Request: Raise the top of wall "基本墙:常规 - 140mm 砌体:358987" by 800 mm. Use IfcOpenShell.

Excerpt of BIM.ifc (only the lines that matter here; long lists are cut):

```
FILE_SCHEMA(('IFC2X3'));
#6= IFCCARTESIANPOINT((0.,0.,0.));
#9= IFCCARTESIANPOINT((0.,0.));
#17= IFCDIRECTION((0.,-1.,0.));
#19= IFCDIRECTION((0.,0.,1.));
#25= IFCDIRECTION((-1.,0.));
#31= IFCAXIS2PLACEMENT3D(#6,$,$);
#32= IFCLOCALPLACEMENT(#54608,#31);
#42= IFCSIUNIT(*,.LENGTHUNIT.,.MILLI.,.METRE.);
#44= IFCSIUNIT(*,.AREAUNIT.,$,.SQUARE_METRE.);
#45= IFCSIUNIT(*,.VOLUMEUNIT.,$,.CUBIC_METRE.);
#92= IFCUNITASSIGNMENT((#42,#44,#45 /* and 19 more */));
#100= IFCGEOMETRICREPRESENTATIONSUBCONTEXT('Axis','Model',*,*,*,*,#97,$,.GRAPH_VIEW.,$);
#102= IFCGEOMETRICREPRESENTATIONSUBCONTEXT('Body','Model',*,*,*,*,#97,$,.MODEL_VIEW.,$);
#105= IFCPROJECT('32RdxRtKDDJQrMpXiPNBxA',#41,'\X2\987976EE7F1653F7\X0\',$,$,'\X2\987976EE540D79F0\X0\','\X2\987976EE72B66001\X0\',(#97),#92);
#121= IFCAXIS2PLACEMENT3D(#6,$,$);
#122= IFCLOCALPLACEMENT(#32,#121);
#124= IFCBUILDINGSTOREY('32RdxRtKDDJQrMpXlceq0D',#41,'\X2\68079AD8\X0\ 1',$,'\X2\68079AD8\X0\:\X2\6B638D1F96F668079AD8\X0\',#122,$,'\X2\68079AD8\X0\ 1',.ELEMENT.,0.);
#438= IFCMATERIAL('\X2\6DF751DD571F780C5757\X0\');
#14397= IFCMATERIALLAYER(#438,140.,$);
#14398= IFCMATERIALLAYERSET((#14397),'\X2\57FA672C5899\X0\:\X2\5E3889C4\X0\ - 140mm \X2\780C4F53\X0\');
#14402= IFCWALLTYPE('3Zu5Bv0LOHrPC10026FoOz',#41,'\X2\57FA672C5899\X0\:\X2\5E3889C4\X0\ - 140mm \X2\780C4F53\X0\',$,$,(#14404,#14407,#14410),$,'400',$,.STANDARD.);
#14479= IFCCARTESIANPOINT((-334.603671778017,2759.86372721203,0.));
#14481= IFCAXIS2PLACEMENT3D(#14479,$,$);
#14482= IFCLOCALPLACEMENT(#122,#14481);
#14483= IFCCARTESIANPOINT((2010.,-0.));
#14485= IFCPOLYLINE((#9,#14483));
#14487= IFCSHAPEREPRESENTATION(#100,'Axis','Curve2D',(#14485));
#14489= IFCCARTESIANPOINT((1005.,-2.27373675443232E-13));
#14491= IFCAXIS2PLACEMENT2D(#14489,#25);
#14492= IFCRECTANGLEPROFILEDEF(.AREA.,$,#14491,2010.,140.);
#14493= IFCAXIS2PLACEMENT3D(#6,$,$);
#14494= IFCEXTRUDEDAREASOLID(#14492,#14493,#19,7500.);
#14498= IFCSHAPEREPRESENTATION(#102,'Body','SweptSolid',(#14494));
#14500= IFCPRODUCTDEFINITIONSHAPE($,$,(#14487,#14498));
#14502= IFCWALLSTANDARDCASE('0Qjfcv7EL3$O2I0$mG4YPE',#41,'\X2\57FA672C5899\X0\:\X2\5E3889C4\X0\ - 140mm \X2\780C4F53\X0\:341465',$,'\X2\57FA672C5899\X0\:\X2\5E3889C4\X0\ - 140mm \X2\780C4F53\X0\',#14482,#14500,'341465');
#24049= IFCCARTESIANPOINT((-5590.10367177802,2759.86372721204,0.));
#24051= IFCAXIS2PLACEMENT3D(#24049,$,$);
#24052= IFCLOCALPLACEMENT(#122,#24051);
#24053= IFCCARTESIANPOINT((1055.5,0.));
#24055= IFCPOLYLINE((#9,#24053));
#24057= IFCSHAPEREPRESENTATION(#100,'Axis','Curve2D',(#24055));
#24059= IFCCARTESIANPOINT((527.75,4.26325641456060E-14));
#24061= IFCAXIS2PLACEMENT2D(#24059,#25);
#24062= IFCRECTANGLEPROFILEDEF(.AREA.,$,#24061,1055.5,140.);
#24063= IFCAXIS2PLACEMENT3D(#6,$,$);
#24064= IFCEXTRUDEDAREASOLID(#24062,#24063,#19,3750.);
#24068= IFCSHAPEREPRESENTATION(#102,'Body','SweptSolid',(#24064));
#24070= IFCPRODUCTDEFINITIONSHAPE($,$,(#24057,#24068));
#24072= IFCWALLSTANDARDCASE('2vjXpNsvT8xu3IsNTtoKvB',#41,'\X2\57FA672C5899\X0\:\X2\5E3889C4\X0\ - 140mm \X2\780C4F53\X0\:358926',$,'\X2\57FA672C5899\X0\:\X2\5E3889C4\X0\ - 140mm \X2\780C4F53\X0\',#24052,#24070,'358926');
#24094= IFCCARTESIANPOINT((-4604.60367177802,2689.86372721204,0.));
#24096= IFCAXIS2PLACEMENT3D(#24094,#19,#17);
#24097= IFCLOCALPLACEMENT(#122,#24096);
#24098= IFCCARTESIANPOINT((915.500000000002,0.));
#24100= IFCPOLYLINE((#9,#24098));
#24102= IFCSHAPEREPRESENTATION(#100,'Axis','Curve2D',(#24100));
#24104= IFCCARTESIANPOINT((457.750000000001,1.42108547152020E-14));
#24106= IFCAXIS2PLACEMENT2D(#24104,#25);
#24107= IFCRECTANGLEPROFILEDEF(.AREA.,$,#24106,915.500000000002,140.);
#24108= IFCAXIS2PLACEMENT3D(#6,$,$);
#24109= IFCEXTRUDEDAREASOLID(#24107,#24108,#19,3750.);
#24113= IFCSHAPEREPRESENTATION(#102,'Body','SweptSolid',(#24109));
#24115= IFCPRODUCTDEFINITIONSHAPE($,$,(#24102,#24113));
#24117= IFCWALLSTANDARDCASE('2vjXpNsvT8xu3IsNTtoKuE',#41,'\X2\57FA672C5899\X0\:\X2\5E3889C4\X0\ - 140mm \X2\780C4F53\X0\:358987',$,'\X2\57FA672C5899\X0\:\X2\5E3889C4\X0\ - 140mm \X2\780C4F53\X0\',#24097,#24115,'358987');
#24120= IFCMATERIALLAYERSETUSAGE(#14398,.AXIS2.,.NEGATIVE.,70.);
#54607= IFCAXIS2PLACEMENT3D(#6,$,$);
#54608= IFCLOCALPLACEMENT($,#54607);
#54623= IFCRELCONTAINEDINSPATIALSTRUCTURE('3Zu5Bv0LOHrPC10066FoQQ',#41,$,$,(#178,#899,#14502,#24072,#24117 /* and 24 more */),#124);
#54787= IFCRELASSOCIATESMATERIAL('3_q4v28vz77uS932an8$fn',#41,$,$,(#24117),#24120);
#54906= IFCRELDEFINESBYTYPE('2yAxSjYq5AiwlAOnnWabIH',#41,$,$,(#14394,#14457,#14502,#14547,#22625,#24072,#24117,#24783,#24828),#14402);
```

```python
import ifcopenshell
import ifcopenshell.geom
import ifcopenshell.util.representation
import ifcopenshell.util.shape

model = ifcopenshell.open("BIM.ifc")
settings = ifcopenshell.geom.settings()


def volume(element):
    """Net volume in cubic metres, openings subtracted."""
    shape = ifcopenshell.geom.create_shape(settings, element)
    return ifcopenshell.util.shape.get_volume(shape.geometry)


wall = model.by_id(24117)
before = volume(wall)

body = ifcopenshell.util.representation.get_representation(wall, "Model", "Body")
solid = body.Items[0]
old_height = solid.Depth
solid.Depth += 800.0
after = volume(wall)

print(f"height {old_height:g} -> {solid.Depth:g}, volume {before:.3f} -> {after:.3f} m3")

model.write("BIM_updated.ifc")
```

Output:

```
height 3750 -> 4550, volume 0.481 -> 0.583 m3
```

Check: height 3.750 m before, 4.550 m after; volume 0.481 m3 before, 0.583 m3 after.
